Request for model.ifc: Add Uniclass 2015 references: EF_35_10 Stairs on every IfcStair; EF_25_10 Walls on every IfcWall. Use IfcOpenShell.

First a look at what the model holds.

```python
import ifcopenshell

model = ifcopenshell.open("model.ifc")
print(model.schema)
print("classifications:", [c.Name for c in model.by_type("IfcClassification")])
for ifc_class in ("IfcDoor", "IfcRoof", "IfcStair", "IfcWall", "IfcWindow"):
    print(ifc_class, len(model.by_type(ifc_class)))
```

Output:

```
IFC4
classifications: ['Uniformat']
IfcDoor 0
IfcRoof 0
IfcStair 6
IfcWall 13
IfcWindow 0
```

```python
import ifcopenshell
import ifcopenshell.api.classification

model = ifcopenshell.open("model.ifc")

system = ifcopenshell.api.classification.add_classification(model, classification="Uniclass 2015")

codes = {
    "IfcStair": ("EF_35_10", "Stairs"),
    "IfcWall": ("EF_25_10", "Walls"),
}
for ifc_class, (code, name) in codes.items():
    products = model.by_type(ifc_class)
    ifcopenshell.api.classification.add_reference(
        model, products=products, classification=system, identification=code, name=name
    )
    print(code, len(products))

model.write("model_updated.ifc")
```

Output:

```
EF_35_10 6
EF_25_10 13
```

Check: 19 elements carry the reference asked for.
